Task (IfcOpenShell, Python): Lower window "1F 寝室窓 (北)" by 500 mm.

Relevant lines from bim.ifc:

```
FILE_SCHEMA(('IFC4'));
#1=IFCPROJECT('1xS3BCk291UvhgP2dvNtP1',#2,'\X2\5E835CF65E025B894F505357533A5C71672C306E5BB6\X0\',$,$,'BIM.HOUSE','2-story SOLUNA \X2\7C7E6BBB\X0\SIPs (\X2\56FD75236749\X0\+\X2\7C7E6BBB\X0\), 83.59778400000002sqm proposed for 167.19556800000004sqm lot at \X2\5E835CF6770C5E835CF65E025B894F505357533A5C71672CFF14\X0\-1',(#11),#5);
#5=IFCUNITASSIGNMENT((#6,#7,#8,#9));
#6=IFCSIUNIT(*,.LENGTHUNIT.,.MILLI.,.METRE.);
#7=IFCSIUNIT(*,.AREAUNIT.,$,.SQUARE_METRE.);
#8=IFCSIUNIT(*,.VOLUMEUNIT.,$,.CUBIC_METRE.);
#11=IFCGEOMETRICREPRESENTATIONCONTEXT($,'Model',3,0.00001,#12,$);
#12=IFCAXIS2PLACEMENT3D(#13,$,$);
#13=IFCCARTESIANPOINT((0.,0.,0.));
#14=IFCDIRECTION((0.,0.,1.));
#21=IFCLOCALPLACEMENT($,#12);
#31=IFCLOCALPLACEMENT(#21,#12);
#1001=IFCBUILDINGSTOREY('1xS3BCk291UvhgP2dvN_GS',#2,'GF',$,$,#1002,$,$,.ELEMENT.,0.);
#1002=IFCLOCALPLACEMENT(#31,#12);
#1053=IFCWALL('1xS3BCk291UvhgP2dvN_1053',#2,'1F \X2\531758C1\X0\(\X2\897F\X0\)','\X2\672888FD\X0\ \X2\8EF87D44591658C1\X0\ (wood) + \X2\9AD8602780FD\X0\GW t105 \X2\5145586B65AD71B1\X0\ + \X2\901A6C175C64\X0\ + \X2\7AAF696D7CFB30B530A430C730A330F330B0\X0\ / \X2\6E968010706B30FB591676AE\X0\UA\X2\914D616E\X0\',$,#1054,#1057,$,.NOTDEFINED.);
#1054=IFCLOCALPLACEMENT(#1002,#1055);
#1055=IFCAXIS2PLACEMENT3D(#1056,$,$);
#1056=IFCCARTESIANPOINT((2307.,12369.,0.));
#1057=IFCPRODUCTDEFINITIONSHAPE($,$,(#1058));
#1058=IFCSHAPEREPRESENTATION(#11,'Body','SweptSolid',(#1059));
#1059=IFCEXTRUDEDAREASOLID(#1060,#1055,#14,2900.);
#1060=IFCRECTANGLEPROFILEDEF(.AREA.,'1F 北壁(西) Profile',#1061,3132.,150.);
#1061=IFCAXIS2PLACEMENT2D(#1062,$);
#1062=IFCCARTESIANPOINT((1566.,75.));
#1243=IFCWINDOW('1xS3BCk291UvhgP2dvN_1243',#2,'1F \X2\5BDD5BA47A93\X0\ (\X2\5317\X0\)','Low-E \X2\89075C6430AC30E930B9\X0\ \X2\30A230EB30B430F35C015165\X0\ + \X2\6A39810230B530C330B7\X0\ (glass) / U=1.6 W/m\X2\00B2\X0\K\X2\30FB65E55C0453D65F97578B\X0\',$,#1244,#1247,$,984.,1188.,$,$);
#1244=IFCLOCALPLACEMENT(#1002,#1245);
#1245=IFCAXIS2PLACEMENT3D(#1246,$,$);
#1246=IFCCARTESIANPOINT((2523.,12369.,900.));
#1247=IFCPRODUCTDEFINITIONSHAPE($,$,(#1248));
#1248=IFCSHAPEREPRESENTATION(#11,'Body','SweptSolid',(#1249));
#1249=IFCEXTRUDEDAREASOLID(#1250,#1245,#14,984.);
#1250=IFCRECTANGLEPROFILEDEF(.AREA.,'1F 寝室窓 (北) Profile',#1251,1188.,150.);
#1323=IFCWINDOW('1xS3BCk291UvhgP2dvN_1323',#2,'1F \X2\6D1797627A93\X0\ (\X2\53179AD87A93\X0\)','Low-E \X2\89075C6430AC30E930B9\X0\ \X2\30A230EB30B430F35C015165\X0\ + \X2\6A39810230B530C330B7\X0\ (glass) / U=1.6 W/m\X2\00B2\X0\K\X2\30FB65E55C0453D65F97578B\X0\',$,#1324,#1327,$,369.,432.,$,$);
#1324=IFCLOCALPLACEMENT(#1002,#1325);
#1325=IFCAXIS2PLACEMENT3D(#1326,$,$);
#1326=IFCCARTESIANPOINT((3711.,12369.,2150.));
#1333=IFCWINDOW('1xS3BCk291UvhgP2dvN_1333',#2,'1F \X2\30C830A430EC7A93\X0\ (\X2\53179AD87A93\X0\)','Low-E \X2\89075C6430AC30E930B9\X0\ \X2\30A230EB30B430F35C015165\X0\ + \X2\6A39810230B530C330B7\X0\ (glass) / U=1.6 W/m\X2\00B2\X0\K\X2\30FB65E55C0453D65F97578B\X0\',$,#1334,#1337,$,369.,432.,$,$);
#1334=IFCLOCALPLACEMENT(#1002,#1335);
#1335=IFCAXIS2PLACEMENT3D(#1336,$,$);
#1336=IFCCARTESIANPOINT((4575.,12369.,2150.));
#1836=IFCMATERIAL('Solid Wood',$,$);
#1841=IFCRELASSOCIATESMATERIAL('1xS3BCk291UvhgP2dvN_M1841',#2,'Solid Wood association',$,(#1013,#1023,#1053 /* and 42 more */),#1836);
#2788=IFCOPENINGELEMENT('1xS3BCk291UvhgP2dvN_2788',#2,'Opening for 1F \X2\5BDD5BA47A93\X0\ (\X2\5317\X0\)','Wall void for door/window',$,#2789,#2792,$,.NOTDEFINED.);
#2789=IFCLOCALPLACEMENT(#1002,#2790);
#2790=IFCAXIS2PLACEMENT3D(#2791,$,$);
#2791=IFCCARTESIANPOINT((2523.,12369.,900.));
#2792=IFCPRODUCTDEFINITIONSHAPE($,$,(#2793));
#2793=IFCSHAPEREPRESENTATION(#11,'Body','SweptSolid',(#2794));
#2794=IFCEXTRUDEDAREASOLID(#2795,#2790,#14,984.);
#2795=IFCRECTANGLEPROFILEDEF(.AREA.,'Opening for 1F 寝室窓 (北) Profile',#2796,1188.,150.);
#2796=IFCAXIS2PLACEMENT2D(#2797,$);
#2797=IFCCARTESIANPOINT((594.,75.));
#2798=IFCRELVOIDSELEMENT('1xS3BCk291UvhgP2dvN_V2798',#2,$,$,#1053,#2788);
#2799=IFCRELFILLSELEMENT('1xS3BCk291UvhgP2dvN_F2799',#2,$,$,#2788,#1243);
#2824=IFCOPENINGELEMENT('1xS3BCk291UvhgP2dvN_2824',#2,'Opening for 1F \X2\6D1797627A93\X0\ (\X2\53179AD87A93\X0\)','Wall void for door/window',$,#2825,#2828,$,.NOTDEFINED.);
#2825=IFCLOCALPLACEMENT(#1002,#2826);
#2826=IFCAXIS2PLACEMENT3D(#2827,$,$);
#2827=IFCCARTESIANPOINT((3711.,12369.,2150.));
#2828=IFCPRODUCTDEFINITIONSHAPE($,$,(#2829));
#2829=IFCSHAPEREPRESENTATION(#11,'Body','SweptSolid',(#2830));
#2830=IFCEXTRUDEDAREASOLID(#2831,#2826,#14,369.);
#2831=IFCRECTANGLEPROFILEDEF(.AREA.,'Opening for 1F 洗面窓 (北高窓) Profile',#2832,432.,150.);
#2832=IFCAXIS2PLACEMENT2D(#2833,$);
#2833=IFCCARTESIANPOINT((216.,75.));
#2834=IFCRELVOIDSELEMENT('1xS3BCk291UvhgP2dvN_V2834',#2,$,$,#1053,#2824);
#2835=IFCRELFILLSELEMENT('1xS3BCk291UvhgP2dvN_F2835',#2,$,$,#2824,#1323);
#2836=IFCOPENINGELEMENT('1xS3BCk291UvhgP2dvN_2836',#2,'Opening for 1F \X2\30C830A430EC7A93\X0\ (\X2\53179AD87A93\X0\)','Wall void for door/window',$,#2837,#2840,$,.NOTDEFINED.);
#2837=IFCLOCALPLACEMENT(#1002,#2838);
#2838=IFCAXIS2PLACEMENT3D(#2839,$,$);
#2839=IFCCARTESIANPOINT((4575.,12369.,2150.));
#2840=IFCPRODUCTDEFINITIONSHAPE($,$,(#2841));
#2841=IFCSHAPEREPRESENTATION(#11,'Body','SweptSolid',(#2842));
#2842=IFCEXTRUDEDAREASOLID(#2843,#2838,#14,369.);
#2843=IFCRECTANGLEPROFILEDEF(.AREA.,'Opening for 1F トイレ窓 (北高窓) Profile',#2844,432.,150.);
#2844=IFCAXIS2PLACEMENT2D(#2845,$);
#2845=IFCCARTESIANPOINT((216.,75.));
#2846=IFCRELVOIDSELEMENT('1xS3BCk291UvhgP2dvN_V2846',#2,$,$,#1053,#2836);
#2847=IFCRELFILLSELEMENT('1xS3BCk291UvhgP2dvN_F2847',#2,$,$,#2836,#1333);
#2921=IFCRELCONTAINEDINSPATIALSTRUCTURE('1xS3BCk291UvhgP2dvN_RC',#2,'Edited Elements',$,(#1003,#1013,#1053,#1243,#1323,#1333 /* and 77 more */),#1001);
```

```python
import numpy as np
import ifcopenshell
import ifcopenshell.api.geometry
import ifcopenshell.util.placement
import ifcopenshell.util.unit

model = ifcopenshell.open("bim.ifc")
unit_scale = ifcopenshell.util.unit.calculate_unit_scale(model)

window = model.by_guid("1xS3BCk291UvhgP2dvN_1243")
opening = window.FillsVoids[0].RelatingOpeningElement
dz = -0.5 / unit_scale

shift = np.array([0.0, 0.0, dz])
# The window is not placed relative to its opening, so move both.
for product in (opening, window):
    matrix = ifcopenshell.util.placement.get_local_placement(product.ObjectPlacement)
    matrix[:3, 3] += shift
    ifcopenshell.api.geometry.edit_object_placement(model, product=product, matrix=matrix, is_si=False)

print(f"moved by {dz * unit_scale:+.3f} m")

model.write("bim_v2.ifc")
```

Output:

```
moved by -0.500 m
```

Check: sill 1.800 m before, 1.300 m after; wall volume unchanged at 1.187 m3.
